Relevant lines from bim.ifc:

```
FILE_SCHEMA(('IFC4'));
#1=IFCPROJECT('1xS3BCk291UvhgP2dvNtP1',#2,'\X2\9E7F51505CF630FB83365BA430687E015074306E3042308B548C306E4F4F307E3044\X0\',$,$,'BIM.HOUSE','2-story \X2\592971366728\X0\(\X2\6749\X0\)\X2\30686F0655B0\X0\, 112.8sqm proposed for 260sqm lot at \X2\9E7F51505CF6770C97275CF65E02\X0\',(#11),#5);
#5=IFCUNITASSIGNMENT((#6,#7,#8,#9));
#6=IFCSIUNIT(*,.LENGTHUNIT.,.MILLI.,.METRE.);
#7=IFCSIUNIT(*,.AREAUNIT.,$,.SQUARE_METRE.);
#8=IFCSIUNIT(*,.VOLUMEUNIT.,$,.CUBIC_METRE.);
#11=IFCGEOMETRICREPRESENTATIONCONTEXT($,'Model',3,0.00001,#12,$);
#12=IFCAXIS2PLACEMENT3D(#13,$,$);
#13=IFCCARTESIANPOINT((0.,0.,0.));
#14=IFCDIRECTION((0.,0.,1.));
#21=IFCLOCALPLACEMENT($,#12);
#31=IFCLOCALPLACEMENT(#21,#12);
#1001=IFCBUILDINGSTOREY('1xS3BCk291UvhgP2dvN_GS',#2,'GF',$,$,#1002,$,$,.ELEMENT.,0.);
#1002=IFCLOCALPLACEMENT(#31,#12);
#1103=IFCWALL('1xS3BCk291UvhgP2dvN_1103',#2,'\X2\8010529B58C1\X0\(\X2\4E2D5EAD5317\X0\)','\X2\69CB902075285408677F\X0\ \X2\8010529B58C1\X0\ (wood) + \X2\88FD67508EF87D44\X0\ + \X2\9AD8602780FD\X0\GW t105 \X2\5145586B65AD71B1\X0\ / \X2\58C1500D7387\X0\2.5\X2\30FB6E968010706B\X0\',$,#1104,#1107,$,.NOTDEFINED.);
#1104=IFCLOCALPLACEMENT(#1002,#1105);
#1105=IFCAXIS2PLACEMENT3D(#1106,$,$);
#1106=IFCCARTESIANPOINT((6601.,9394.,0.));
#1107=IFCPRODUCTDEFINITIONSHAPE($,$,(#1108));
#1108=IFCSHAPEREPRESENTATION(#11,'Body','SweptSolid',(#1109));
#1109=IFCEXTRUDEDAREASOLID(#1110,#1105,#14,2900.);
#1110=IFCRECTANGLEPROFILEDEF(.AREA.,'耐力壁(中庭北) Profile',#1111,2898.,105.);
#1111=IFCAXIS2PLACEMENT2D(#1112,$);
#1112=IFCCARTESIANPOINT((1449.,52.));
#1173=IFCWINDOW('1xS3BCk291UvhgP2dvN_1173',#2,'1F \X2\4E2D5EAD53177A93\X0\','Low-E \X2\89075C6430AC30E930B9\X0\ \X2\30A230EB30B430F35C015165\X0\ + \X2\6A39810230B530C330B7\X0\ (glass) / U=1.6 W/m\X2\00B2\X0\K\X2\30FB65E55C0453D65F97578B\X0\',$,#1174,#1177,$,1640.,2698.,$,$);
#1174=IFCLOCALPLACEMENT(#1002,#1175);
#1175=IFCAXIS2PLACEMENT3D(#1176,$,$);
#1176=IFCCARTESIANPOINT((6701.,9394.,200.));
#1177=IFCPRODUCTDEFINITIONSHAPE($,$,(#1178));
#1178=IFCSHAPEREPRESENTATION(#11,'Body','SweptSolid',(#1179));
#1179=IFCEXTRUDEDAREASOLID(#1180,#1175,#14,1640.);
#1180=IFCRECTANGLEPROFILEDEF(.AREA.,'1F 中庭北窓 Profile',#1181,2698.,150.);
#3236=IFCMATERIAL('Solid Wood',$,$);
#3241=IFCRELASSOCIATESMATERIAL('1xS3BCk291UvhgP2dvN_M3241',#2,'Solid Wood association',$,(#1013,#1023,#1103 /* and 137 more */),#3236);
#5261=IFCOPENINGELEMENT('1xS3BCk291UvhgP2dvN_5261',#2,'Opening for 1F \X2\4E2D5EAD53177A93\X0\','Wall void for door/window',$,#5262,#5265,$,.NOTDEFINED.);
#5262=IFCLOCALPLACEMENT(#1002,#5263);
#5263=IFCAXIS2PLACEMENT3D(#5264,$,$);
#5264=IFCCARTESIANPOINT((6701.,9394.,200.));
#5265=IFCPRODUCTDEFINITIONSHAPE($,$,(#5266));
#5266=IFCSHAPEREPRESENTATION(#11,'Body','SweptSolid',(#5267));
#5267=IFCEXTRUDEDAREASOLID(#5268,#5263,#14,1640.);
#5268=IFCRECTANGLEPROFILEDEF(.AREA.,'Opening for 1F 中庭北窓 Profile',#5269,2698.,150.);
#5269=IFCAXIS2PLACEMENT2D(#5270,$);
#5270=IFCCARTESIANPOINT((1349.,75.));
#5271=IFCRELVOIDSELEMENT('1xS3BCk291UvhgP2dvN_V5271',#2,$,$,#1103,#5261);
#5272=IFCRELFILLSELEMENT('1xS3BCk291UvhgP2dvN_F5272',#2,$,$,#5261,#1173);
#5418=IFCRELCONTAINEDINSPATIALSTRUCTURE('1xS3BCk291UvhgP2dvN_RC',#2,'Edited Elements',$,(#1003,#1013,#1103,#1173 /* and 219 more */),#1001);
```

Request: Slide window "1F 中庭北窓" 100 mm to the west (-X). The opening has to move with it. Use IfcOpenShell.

```python
import ifcopenshell
import ifcopenshell.api.geometry
import ifcopenshell.util.placement
import ifcopenshell.util.unit

model = ifcopenshell.open("bim.ifc")
unit_scale = ifcopenshell.util.unit.calculate_unit_scale(model)

window = model.by_guid("1xS3BCk291UvhgP2dvN_1173")
opening = window.FillsVoids[0].RelatingOpeningElement
wall = opening.VoidsElements[0].RelatingBuildingElement

wall_matrix = ifcopenshell.util.placement.get_local_placement(wall.ObjectPlacement)
shift = wall_matrix[:3, 0] * -0.1 / unit_scale
before = ifcopenshell.util.placement.get_local_placement(window.ObjectPlacement)[:3, 3].copy()

# The window is not placed relative to its opening, so move both.
for product in (opening, window):
    matrix = ifcopenshell.util.placement.get_local_placement(product.ObjectPlacement)
    matrix[:3, 3] += shift
    ifcopenshell.api.geometry.edit_object_placement(model, product=product, matrix=matrix, is_si=False)

after = ifcopenshell.util.placement.get_local_placement(window.ObjectPlacement)[:3, 3]
print("window moved by", (after - before).round(3) + 0.0)

model.write("bim_rev.ifc")
```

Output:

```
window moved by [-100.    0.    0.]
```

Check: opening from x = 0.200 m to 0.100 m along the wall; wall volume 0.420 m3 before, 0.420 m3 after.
